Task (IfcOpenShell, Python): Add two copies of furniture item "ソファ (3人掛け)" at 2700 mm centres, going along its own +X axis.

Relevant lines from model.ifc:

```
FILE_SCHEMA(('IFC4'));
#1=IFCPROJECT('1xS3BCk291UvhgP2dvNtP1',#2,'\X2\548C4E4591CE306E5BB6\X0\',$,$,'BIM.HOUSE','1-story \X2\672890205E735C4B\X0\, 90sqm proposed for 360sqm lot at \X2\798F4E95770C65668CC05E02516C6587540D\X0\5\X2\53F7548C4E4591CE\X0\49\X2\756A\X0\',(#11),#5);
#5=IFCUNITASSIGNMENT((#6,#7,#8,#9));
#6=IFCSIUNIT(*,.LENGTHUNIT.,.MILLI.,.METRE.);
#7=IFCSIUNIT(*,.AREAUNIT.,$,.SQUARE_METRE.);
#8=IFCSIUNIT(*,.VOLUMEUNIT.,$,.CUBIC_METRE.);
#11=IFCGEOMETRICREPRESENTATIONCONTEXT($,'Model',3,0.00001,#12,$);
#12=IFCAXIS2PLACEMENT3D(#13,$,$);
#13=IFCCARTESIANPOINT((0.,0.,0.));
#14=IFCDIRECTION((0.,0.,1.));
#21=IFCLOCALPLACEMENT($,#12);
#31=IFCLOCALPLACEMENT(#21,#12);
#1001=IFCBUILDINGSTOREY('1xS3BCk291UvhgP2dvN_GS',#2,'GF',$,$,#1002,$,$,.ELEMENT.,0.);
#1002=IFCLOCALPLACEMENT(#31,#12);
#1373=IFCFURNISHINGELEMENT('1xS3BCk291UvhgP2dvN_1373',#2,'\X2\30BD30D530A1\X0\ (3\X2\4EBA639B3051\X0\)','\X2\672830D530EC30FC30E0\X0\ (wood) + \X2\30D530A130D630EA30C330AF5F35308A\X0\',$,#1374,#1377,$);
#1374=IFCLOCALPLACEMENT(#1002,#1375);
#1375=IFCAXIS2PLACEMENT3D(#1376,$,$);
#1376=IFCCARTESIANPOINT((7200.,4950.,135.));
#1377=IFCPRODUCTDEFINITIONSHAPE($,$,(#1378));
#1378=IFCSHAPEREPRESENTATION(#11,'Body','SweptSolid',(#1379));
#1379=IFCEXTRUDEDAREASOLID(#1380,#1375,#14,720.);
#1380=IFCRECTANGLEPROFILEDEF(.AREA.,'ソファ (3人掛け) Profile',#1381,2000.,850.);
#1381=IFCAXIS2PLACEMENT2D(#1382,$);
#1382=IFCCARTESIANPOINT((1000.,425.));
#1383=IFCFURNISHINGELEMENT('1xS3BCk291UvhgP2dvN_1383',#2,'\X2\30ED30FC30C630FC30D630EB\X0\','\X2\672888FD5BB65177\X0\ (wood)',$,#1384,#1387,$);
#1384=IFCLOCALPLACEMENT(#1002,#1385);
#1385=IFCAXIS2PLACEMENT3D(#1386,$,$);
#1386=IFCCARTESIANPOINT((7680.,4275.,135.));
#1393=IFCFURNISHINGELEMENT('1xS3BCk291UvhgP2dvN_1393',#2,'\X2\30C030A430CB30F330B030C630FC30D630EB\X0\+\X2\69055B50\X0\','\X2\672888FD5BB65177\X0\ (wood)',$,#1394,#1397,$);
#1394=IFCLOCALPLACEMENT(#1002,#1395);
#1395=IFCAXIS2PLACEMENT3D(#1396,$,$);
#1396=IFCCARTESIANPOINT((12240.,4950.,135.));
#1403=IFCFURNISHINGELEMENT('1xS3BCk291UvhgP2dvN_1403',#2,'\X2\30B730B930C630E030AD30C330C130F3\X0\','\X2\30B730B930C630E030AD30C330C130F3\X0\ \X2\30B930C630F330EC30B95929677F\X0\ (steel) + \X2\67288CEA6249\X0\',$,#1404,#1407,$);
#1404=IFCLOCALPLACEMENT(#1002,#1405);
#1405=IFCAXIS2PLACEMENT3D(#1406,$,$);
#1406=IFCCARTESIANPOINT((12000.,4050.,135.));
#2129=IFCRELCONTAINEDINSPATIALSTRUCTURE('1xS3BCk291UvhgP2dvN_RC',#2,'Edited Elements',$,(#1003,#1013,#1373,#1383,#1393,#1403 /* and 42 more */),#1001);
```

```python
import ifcopenshell
import ifcopenshell.api.geometry
import ifcopenshell.api.root
import ifcopenshell.util.element
import ifcopenshell.util.placement

model = ifcopenshell.open("model.ifc")


def reuse_history(source, copy):
    """copy_class also copies each property set's owner history, people and application; keep the originals."""
    for rel in copy.IsDefinedBy:
        if rel.is_a("IfcRelDefinesByProperties") and (history := rel.RelatingPropertyDefinition.OwnerHistory):
            rel.RelatingPropertyDefinition.OwnerHistory = source.OwnerHistory
            ifcopenshell.util.element.remove_deep2(model, history)


source = model.by_guid("1xS3BCk291UvhgP2dvN_1373")
base = ifcopenshell.util.placement.get_local_placement(source.ObjectPlacement)
step = base[:3, 0] * 2700.0

for i in range(1, 3):
    copy = ifcopenshell.api.root.copy_class(model, product=source)
    copy.Representation = ifcopenshell.util.element.copy_deep(
        model, source.Representation, exclude=["IfcGeometricRepresentationContext", "IfcRepresentationMap"]
    )
    reuse_history(source, copy)
    matrix = base.copy()
    matrix[:3, 3] += i * step
    print("added at", matrix[:3, 3].round(3) + 0.0)
    ifcopenshell.api.geometry.edit_object_placement(model, product=copy, matrix=matrix, is_si=False)

model.write("model_updated.ifc")
```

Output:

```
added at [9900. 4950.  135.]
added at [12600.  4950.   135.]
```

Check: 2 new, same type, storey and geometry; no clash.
